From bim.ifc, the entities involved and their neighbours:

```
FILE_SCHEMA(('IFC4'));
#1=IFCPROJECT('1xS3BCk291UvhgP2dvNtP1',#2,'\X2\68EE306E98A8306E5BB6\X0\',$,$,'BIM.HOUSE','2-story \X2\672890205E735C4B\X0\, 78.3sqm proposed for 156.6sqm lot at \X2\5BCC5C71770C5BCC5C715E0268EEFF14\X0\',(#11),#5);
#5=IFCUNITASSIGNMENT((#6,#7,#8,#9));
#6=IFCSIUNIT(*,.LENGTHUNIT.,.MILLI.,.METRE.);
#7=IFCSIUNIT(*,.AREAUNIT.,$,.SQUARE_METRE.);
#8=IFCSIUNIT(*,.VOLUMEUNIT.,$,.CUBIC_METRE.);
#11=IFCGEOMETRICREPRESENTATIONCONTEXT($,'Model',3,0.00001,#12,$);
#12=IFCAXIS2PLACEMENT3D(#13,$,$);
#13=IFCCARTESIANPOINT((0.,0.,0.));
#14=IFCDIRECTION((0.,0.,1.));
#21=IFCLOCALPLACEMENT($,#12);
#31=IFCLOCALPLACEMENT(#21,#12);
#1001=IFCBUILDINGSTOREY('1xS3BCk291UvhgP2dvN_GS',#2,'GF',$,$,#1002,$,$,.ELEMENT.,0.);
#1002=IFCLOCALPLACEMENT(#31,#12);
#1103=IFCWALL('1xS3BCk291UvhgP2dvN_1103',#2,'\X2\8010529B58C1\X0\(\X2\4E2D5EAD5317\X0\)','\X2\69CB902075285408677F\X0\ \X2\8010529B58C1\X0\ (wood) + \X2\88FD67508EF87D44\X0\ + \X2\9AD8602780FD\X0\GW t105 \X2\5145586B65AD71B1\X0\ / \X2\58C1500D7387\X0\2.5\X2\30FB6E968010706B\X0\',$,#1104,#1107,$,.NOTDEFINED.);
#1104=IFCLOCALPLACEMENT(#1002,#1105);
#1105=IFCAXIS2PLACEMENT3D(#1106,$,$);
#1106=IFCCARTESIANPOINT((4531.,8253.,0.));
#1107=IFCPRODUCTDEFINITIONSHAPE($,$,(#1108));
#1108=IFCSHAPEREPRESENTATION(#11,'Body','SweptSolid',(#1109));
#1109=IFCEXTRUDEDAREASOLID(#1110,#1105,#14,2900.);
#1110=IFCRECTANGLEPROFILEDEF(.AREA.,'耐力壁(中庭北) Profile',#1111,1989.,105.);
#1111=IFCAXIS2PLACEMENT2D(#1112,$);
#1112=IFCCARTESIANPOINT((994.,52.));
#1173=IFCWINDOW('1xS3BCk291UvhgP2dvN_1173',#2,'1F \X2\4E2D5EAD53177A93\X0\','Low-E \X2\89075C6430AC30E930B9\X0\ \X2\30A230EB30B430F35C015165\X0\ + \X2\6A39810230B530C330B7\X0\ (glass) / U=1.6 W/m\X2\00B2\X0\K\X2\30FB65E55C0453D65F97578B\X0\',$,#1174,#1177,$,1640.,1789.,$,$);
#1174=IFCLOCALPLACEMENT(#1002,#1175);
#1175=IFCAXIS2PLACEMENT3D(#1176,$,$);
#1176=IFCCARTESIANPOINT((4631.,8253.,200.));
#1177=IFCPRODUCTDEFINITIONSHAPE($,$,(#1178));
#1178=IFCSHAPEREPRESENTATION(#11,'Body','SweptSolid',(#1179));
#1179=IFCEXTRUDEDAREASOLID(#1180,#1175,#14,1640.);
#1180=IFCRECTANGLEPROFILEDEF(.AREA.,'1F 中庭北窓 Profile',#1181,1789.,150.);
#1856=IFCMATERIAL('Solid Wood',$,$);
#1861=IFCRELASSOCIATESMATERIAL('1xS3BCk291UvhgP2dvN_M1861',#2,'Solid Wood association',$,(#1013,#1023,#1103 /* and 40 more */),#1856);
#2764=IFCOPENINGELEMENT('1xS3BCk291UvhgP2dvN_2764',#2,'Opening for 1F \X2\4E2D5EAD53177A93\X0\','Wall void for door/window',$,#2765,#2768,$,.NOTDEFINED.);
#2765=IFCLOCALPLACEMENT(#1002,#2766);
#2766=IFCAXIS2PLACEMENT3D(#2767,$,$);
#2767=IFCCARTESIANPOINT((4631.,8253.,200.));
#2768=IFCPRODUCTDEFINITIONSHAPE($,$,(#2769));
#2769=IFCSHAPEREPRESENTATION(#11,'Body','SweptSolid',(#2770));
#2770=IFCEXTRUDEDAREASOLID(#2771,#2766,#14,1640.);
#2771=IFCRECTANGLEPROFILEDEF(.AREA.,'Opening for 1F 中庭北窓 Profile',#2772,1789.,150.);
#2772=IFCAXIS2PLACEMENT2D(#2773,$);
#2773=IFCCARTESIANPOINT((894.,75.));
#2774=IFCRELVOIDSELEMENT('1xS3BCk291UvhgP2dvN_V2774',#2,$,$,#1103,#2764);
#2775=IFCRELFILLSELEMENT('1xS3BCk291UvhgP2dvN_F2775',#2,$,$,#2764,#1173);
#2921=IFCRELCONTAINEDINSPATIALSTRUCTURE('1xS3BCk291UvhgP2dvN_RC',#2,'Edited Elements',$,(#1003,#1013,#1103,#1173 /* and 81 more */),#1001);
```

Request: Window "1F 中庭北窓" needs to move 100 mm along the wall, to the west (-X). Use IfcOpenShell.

```python
import ifcopenshell
import ifcopenshell.api.geometry
import ifcopenshell.util.placement

model = ifcopenshell.open("bim.ifc")

window = model.by_id(1173)
opening = window.FillsVoids[0].RelatingOpeningElement
wall = opening.VoidsElements[0].RelatingBuildingElement

wall_matrix = ifcopenshell.util.placement.get_local_placement(wall.ObjectPlacement)
shift = wall_matrix[:3, 0] * -100.0
before = ifcopenshell.util.placement.get_local_placement(window.ObjectPlacement)[:3, 3].copy()

# The window is not placed relative to its opening, so move both.
for product in (opening, window):
    matrix = ifcopenshell.util.placement.get_local_placement(product.ObjectPlacement)
    matrix[:3, 3] += shift
    ifcopenshell.api.geometry.edit_object_placement(model, product=product, matrix=matrix, is_si=False)

after = ifcopenshell.util.placement.get_local_placement(window.ObjectPlacement)[:3, 3]
print("window moved by", (after - before).round(3) + 0.0)

model.write("bim_updated.ifc")
```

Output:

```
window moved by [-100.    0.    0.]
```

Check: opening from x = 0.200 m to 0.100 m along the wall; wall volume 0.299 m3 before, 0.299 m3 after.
